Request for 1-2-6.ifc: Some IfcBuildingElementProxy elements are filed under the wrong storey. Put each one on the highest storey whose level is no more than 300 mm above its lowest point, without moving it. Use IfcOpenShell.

First a look at what the model holds.

```python
import ifcopenshell
import ifcopenshell.util.element
import ifcopenshell.util.placement

model = ifcopenshell.open("1-2-6.ifc")
print(model.schema)
for storey in model.by_type("IfcBuildingStorey"):
    level = ifcopenshell.util.placement.get_storey_elevation(storey)
    count = sum(e.is_a("IfcBuildingElementProxy") for e in ifcopenshell.util.element.get_contained(storey))
    print(storey.id(), storey.Name, round(level, 3), count, sep=" | ")
```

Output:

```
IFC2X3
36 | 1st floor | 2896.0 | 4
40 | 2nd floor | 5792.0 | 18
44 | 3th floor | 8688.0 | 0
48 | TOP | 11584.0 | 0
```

```python
import ifcopenshell
import ifcopenshell.api.spatial
import ifcopenshell.geom
import ifcopenshell.util.element
import ifcopenshell.util.placement
import ifcopenshell.util.shape
import ifcopenshell.util.unit

model = ifcopenshell.open("1-2-6.ifc")
unit_scale = ifcopenshell.util.unit.calculate_unit_scale(model)
settings = ifcopenshell.geom.settings()

levels = sorted(
    ((ifcopenshell.util.placement.get_storey_elevation(s) * unit_scale, s) for s in model.by_type("IfcBuildingStorey")),
    key=lambda pair: pair[0],
)

for e in model.by_type("IfcBuildingElementProxy"):
    current = e.ContainedInStructure[0].RelatingStructure if e.ContainedInStructure else None
    if current is None or not current.is_a("IfcBuildingStorey"):
        continue
    shape = ifcopenshell.geom.create_shape(settings, e)
    bottom = ifcopenshell.util.shape.get_shape_bottom_elevation(shape, shape.geometry)
    below = [s for level, s in levels if level <= bottom + 0.3]
    storey = below[-1] if below else levels[0][1]
    if storey != current:
        # assign_container keeps the world position.
        ifcopenshell.api.spatial.assign_container(model, products=[e], relating_structure=storey)
        print(e.id(), current.Name, "->", storey.Name)

model.write("1-2-6-out.ifc")
```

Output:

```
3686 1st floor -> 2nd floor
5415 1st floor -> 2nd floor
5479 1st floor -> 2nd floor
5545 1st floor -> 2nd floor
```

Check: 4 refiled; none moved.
